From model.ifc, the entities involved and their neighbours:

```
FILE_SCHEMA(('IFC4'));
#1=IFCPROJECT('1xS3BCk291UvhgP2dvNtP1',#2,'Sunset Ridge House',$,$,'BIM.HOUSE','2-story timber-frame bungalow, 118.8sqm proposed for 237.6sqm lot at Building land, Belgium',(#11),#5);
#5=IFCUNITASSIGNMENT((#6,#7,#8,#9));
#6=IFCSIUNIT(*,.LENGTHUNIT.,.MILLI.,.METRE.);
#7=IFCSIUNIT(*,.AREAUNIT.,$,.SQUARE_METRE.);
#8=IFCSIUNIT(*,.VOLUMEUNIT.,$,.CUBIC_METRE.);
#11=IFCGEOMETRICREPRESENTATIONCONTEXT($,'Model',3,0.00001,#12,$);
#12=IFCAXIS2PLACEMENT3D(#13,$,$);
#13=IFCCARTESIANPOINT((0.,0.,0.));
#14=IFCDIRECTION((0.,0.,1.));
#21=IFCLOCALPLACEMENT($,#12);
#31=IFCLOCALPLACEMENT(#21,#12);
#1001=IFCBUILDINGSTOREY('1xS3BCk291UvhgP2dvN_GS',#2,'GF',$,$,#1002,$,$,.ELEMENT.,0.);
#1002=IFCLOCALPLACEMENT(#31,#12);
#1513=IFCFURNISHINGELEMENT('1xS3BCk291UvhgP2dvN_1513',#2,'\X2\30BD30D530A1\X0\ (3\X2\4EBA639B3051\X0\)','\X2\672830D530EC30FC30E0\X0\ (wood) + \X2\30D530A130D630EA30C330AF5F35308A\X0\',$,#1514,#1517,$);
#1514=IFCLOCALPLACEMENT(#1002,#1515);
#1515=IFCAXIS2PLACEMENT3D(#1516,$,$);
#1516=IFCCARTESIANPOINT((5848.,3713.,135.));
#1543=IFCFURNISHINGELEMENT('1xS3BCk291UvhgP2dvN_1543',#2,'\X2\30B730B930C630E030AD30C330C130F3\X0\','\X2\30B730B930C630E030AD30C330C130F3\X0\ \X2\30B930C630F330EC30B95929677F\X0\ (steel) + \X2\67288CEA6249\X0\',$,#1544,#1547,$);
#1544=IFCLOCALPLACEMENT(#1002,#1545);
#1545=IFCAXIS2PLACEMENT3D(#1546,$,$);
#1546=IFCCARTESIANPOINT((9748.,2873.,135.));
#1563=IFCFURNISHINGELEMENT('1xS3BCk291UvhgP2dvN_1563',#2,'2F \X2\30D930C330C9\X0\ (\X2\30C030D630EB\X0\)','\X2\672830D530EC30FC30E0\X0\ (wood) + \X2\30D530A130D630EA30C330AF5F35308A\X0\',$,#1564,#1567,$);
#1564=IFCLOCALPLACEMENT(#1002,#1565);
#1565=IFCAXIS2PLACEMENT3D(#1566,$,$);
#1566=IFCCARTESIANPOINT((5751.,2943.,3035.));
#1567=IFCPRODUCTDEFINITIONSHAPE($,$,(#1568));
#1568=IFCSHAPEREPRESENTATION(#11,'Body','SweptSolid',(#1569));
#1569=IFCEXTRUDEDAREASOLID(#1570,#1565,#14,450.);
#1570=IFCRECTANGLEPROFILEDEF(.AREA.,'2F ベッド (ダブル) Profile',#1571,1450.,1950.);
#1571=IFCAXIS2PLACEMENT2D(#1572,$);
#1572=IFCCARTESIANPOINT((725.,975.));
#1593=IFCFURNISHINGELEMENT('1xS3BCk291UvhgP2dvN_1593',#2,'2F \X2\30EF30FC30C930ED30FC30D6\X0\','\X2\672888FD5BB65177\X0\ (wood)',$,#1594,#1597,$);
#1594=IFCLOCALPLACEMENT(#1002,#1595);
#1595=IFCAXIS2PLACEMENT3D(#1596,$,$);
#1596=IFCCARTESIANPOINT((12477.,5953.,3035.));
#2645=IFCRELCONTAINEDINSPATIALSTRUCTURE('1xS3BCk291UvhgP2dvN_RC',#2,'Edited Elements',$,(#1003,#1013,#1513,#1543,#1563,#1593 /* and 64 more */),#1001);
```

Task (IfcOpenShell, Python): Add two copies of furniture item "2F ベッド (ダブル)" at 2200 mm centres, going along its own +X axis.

```python
import ifcopenshell
import ifcopenshell.api.geometry
import ifcopenshell.api.root
import ifcopenshell.util.element
import ifcopenshell.util.placement
import ifcopenshell.util.unit

model = ifcopenshell.open("model.ifc")
unit_scale = ifcopenshell.util.unit.calculate_unit_scale(model)


def reuse_history(source, copy):
    """copy_class also copies each property set's owner history, people and application; keep the originals."""
    for rel in copy.IsDefinedBy:
        if rel.is_a("IfcRelDefinesByProperties") and (history := rel.RelatingPropertyDefinition.OwnerHistory):
            rel.RelatingPropertyDefinition.OwnerHistory = source.OwnerHistory
            ifcopenshell.util.element.remove_deep2(model, history)


source = model.by_guid("1xS3BCk291UvhgP2dvN_1563")
base = ifcopenshell.util.placement.get_local_placement(source.ObjectPlacement)
step = base[:3, 0] * 2.2 / unit_scale

for i in range(1, 3):
    copy = ifcopenshell.api.root.copy_class(model, product=source)
    copy.Representation = ifcopenshell.util.element.copy_deep(
        model, source.Representation, exclude=["IfcGeometricRepresentationContext", "IfcRepresentationMap"]
    )
    reuse_history(source, copy)
    matrix = base.copy()
    matrix[:3, 3] += i * step
    print("added at", matrix[:3, 3].round(3) + 0.0)
    ifcopenshell.api.geometry.edit_object_placement(model, product=copy, matrix=matrix, is_si=False)

model.write("model_rev.ifc")
```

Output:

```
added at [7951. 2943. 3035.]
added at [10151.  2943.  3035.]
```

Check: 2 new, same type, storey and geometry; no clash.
